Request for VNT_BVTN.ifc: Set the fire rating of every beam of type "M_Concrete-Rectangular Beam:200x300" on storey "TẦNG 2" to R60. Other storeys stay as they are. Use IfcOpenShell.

First a look at what the model holds.

```python
import ifcopenshell
import ifcopenshell.util.element

model = ifcopenshell.open("VNT_BVTN.ifc")
print(model.schema)
storey = next(s for s in model.by_type("IfcBuildingStorey") if s.Name == "TẦNG 2")
beams = [e for e in ifcopenshell.util.element.get_decomposition(storey) if e.is_a("IfcBeam")]
seen = {}
for e in beams:
    element_type = ifcopenshell.util.element.get_type(e)
    key = (element_type.Name if element_type != e and element_type else None, ifcopenshell.util.element.get_pset(e, "Pset_BeamCommon", "FireRating"))
    seen[key] = seen.get(key, 0) + 1
for (name, value), count in sorted(seen.items(), key=str):
    print(count, "x", name, "|", value)
```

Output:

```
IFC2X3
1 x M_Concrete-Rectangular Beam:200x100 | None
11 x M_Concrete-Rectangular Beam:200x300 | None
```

```python
import ifcopenshell
import ifcopenshell.api.pset
import ifcopenshell.util.element

model = ifcopenshell.open("VNT_BVTN.ifc")

storey = next(s for s in model.by_type("IfcBuildingStorey") if s.Name == "TẦNG 2")
beams = [e for e in ifcopenshell.util.element.get_decomposition(storey) if e.is_a("IfcBeam")]

count = 0
for e in beams:
    element_type = ifcopenshell.util.element.get_type(e)
    if element_type in (None, e) or element_type.Name != "M_Concrete-Rectangular Beam:200x300":
        continue
    # add_pset returns the element's existing set when there is one.
    pset = ifcopenshell.api.pset.add_pset(model, product=e, name="Pset_BeamCommon")
    ifcopenshell.api.pset.edit_pset(model, pset=pset, properties={"FireRating": "R60"})
    count += 1

print(count, "beams updated")

model.write("VNT_BVTN_updated.ifc")
```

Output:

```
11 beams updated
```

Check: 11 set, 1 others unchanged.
